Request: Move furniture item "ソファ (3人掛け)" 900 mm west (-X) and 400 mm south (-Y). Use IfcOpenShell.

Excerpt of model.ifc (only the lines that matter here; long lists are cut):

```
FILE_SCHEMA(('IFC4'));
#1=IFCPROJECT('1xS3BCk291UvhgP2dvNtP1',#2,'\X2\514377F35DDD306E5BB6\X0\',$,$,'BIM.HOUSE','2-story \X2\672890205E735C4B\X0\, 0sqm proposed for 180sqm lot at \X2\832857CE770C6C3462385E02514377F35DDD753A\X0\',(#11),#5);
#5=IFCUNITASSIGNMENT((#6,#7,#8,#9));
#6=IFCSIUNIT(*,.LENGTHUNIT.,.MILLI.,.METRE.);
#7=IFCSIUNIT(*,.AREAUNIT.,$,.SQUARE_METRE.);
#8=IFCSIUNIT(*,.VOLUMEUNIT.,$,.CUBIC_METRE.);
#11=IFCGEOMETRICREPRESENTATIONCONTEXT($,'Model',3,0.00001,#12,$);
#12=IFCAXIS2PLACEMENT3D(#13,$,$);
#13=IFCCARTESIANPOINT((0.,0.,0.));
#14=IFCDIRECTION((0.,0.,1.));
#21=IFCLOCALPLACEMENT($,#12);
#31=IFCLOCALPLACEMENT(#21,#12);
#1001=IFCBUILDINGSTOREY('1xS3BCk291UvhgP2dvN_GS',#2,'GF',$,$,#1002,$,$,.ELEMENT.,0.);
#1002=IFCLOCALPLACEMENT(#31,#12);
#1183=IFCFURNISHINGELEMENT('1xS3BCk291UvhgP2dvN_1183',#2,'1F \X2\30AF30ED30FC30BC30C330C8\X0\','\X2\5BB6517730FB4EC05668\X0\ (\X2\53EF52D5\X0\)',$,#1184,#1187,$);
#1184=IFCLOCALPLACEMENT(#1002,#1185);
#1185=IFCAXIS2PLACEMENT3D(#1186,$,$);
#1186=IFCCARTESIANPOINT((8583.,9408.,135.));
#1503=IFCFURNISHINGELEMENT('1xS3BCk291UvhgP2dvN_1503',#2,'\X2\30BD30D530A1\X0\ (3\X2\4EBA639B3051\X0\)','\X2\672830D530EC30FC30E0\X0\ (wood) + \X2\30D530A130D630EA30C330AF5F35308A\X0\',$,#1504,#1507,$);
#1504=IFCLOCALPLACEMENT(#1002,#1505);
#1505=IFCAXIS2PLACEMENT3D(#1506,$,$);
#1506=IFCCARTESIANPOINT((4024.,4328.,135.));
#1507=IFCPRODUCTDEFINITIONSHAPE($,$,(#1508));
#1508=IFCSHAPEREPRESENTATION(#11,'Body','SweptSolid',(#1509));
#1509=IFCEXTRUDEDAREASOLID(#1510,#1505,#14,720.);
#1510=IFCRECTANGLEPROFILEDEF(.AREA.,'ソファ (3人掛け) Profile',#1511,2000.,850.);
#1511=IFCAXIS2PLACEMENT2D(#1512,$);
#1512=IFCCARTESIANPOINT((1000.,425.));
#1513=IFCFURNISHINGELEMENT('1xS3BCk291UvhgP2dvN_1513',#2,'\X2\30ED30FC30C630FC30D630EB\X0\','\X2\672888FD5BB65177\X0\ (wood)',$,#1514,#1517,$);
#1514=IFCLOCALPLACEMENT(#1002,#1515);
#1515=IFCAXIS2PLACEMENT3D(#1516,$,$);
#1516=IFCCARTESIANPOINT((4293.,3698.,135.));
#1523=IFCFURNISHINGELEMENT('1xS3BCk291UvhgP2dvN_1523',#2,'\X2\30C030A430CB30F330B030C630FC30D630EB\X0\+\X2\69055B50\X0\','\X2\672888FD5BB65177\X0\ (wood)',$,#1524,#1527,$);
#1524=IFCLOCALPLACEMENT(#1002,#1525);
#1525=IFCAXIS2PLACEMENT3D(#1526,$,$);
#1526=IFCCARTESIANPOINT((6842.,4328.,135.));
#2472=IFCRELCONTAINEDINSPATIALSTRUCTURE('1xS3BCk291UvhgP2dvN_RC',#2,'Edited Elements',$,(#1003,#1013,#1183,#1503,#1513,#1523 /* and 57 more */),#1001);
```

```python
import ifcopenshell
import ifcopenshell.api.geometry
import ifcopenshell.util.placement
import ifcopenshell.util.unit

model = ifcopenshell.open("model.ifc")
unit_scale = ifcopenshell.util.unit.calculate_unit_scale(model)

item = model.by_guid("1xS3BCk291UvhgP2dvN_1503")
matrix = ifcopenshell.util.placement.get_local_placement(item.ObjectPlacement)
matrix[0, 3] -= 0.9 / unit_scale
matrix[1, 3] -= 0.4 / unit_scale
ifcopenshell.api.geometry.edit_object_placement(model, product=item, matrix=matrix, is_si=False)

print(ifcopenshell.util.placement.get_local_placement(item.ObjectPlacement).round(3) + 0.0)

model.write("model_updated.ifc")
```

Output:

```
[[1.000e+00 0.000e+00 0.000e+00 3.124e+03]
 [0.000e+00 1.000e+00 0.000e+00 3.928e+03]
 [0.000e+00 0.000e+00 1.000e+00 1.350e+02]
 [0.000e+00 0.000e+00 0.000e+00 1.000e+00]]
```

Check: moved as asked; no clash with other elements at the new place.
